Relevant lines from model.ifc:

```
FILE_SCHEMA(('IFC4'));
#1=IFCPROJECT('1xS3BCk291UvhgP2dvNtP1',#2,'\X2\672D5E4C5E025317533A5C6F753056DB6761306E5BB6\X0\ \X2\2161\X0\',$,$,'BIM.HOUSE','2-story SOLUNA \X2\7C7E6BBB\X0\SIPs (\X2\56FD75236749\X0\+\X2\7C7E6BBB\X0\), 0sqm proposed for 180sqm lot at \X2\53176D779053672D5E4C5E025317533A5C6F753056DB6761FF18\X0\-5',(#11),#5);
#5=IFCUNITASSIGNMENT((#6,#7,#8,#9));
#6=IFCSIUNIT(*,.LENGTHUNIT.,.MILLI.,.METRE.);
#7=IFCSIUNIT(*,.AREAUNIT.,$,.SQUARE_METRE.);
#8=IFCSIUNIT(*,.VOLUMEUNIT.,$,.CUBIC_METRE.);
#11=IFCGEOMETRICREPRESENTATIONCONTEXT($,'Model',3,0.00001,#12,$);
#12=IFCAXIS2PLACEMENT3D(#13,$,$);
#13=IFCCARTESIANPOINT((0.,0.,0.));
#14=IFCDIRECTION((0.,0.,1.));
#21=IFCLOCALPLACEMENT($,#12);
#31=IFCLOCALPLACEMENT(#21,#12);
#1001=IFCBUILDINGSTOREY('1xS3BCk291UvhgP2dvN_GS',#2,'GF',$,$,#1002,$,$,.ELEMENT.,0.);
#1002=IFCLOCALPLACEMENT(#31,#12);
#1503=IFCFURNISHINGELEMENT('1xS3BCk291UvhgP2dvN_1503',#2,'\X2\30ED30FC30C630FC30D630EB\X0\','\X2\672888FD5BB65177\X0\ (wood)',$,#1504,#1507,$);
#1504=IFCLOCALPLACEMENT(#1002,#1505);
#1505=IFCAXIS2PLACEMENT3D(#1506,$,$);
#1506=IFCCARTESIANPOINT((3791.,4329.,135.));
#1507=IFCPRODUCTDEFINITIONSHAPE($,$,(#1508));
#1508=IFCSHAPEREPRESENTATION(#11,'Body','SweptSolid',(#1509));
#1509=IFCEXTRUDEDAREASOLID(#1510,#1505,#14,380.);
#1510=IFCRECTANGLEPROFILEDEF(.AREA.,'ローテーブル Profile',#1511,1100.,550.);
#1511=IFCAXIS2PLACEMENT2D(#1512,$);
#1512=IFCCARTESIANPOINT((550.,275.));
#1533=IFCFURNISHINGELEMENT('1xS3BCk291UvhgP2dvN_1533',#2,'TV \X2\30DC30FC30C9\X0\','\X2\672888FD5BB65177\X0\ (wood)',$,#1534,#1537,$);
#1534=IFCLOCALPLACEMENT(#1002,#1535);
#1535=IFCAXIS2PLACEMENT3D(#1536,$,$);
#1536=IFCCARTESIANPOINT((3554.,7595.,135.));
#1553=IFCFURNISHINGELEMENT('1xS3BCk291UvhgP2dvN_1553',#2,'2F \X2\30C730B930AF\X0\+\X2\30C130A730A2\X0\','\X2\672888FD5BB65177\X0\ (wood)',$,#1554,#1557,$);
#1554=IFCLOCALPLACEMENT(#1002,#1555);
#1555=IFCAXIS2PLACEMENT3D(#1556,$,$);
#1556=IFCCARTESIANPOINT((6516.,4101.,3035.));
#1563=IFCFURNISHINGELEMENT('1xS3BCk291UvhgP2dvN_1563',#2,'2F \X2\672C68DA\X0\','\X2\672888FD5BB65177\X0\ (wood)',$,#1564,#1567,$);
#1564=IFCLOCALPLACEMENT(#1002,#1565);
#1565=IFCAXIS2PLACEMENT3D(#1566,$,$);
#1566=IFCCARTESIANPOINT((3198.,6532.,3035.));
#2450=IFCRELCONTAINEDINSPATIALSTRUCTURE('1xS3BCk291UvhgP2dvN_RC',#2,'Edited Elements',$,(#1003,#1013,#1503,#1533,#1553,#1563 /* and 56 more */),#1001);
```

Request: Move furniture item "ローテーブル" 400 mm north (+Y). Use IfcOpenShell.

```python
import ifcopenshell
import ifcopenshell.api.geometry
import ifcopenshell.util.placement

model = ifcopenshell.open("model.ifc")

item = model.by_guid("1xS3BCk291UvhgP2dvN_1503")
matrix = ifcopenshell.util.placement.get_local_placement(item.ObjectPlacement)
matrix[1, 3] += 400.0
ifcopenshell.api.geometry.edit_object_placement(model, product=item, matrix=matrix, is_si=False)

print(ifcopenshell.util.placement.get_local_placement(item.ObjectPlacement).round(3) + 0.0)

model.write("model_rev.ifc")
```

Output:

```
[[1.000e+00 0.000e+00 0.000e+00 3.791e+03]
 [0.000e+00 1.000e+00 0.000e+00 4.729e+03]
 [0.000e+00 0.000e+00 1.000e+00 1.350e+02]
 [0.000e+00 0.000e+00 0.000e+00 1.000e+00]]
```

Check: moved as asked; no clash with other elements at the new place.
